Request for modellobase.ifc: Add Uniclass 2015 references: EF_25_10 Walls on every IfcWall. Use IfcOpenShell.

First a look at what the model holds.

```python
import ifcopenshell

model = ifcopenshell.open("modellobase.ifc")
print(model.schema)
print("classifications:", [c.Name for c in model.by_type("IfcClassification")])
for ifc_class in ("IfcDoor", "IfcRoof", "IfcStair", "IfcWall", "IfcWindow"):
    print(ifc_class, len(model.by_type(ifc_class)))
```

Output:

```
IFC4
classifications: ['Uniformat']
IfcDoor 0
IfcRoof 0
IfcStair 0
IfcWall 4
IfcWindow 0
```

```python
import ifcopenshell
import ifcopenshell.api.classification

model = ifcopenshell.open("modellobase.ifc")

system = ifcopenshell.api.classification.add_classification(model, classification="Uniclass 2015")

codes = {
    "IfcWall": ("EF_25_10", "Walls"),
}
for ifc_class, (code, name) in codes.items():
    products = model.by_type(ifc_class)
    ifcopenshell.api.classification.add_reference(
        model, products=products, classification=system, identification=code, name=name
    )
    print(code, len(products))

model.write("modellobase_v2.ifc")
```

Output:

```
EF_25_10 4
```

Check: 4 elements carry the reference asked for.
